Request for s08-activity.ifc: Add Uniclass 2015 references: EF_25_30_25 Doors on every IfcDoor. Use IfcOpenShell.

First a look at what the model holds.

```python
import ifcopenshell

model = ifcopenshell.open("s08-activity.ifc")
print(model.schema)
print("classifications:", [c.Name for c in model.by_type("IfcClassification")])
for ifc_class in ("IfcDoor", "IfcRoof", "IfcStair", "IfcWall", "IfcWindow"):
    print(ifc_class, len(model.by_type(ifc_class)))
```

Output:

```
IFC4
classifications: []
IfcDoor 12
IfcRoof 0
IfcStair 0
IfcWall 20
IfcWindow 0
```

```python
import ifcopenshell
import ifcopenshell.api.classification

model = ifcopenshell.open("s08-activity.ifc")

system = ifcopenshell.api.classification.add_classification(model, classification="Uniclass 2015")

codes = {
    "IfcDoor": ("EF_25_30_25", "Doors"),
}
for ifc_class, (code, name) in codes.items():
    products = model.by_type(ifc_class)
    ifcopenshell.api.classification.add_reference(
        model, products=products, classification=system, identification=code, name=name
    )
    print(code, len(products))

model.write("s08-activity_rev.ifc")
```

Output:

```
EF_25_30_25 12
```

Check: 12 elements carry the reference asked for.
